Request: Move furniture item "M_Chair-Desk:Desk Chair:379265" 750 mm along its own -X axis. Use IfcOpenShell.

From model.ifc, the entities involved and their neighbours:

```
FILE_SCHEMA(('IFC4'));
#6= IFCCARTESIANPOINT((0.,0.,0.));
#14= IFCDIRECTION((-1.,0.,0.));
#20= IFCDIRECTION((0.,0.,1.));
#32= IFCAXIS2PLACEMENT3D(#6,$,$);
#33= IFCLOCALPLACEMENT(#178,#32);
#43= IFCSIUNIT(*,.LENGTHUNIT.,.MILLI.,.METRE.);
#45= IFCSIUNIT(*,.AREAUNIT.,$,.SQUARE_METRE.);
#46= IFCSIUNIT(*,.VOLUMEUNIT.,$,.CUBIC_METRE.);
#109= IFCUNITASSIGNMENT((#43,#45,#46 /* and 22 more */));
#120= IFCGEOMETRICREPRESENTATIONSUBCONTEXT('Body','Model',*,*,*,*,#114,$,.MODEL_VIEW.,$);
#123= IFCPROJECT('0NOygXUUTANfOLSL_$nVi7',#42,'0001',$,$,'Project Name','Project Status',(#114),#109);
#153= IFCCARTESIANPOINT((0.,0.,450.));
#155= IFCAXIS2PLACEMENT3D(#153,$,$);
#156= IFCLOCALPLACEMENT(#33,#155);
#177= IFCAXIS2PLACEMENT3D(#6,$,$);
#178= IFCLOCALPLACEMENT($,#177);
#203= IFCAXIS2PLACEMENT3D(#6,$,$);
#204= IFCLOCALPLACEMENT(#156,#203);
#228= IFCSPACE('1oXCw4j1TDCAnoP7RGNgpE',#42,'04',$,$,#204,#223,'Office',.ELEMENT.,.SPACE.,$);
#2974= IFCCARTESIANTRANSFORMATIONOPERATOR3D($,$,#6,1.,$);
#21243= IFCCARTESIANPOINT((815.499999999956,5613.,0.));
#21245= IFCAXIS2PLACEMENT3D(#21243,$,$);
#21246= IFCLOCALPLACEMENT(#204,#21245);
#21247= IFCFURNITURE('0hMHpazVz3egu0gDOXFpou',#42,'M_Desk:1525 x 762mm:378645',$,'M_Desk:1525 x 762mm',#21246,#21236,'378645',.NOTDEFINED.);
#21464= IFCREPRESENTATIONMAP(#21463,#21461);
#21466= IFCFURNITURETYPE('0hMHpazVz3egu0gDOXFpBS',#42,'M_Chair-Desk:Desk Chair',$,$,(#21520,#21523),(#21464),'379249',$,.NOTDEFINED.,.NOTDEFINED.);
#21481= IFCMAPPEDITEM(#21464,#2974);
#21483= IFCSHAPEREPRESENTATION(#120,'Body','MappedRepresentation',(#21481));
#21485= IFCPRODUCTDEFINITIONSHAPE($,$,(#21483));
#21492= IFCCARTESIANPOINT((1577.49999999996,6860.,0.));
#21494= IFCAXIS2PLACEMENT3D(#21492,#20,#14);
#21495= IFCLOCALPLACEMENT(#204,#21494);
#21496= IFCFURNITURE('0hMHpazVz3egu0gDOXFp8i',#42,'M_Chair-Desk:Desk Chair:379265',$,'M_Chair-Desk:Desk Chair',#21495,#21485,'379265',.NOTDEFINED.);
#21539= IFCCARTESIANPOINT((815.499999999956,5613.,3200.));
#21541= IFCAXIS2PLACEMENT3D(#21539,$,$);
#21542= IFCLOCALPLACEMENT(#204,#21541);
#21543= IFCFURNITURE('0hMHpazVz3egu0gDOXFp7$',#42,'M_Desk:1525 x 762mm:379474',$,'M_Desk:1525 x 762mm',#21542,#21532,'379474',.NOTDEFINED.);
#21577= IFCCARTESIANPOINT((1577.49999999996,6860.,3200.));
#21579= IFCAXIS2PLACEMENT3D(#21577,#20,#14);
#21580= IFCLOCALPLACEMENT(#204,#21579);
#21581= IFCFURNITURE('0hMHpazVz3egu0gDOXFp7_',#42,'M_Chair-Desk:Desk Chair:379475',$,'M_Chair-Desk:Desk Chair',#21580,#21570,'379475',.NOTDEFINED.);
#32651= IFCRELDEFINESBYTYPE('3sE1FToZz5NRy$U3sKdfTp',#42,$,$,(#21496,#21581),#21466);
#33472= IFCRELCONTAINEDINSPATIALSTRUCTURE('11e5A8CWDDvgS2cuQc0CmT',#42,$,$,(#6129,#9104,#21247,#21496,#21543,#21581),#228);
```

```python
import ifcopenshell
import ifcopenshell.api.geometry
import ifcopenshell.util.placement

model = ifcopenshell.open("model.ifc")

item = model.by_id(21496)
matrix = ifcopenshell.util.placement.get_local_placement(item.ObjectPlacement)
matrix[:3, 3] -= matrix[:3, 0] * 750.0
ifcopenshell.api.geometry.edit_object_placement(model, product=item, matrix=matrix, is_si=False)

print(ifcopenshell.util.placement.get_local_placement(item.ObjectPlacement).round(3) + 0.0)

model.write("model-out.ifc")
```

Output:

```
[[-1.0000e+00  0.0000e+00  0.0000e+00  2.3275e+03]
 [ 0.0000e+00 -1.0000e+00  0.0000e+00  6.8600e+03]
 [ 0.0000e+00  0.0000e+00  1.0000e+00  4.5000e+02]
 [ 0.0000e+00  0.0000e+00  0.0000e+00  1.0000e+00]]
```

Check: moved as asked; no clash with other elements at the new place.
